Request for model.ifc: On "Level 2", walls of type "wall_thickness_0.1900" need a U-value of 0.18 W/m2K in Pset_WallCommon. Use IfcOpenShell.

First a look at what the model holds.

```python
import ifcopenshell
import ifcopenshell.util.element

model = ifcopenshell.open("model.ifc")
print(model.schema)
storey = next(s for s in model.by_type("IfcBuildingStorey") if s.Name == "Level 2")
walls = [e for e in ifcopenshell.util.element.get_decomposition(storey) if e.is_a("IfcWall")]
seen = {}
for e in walls:
    element_type = ifcopenshell.util.element.get_type(e)
    key = (element_type.Name if element_type != e and element_type else None, ifcopenshell.util.element.get_pset(e, "Pset_WallCommon", "ThermalTransmittance"))
    seen[key] = seen.get(key, 0) + 1
for (name, value), count in sorted(seen.items(), key=str):
    print(count, "x", name, "|", value)
```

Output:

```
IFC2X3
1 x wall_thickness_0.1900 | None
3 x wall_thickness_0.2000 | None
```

```python
import ifcopenshell
import ifcopenshell.api.pset
import ifcopenshell.util.element

model = ifcopenshell.open("model.ifc")

storey = next(s for s in model.by_type("IfcBuildingStorey") if s.Name == "Level 2")
walls = [e for e in ifcopenshell.util.element.get_decomposition(storey) if e.is_a("IfcWall")]

count = 0
for e in walls:
    element_type = ifcopenshell.util.element.get_type(e)
    if element_type in (None, e) or element_type.Name != "wall_thickness_0.1900":
        continue
    # add_pset returns the element's existing set when there is one.
    pset = ifcopenshell.api.pset.add_pset(model, product=e, name="Pset_WallCommon")
    ifcopenshell.api.pset.edit_pset(model, pset=pset, properties={"ThermalTransmittance": 0.18})
    count += 1

print(count, "walls updated")

model.write("model_edited.ifc")
```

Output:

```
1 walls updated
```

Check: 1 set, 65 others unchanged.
